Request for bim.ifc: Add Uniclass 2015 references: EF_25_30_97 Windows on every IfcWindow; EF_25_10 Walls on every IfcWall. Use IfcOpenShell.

First a look at what the model holds.

```python
import ifcopenshell

model = ifcopenshell.open("bim.ifc")
print(model.schema)
print("classifications:", [c.Name for c in model.by_type("IfcClassification")])
for ifc_class in ("IfcDoor", "IfcRoof", "IfcStair", "IfcWall", "IfcWindow"):
    print(ifc_class, len(model.by_type(ifc_class)))
```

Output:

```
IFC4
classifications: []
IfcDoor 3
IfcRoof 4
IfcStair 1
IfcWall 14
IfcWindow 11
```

```python
import ifcopenshell
import ifcopenshell.api.classification

model = ifcopenshell.open("bim.ifc")

system = ifcopenshell.api.classification.add_classification(model, classification="Uniclass 2015")

codes = {
    "IfcWindow": ("EF_25_30_97", "Windows"),
    "IfcWall": ("EF_25_10", "Walls"),
}
for ifc_class, (code, name) in codes.items():
    products = model.by_type(ifc_class)
    ifcopenshell.api.classification.add_reference(
        model, products=products, classification=system, identification=code, name=name
    )
    print(code, len(products))

model.write("bim-out.ifc")
```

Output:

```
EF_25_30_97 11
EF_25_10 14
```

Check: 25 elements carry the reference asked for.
